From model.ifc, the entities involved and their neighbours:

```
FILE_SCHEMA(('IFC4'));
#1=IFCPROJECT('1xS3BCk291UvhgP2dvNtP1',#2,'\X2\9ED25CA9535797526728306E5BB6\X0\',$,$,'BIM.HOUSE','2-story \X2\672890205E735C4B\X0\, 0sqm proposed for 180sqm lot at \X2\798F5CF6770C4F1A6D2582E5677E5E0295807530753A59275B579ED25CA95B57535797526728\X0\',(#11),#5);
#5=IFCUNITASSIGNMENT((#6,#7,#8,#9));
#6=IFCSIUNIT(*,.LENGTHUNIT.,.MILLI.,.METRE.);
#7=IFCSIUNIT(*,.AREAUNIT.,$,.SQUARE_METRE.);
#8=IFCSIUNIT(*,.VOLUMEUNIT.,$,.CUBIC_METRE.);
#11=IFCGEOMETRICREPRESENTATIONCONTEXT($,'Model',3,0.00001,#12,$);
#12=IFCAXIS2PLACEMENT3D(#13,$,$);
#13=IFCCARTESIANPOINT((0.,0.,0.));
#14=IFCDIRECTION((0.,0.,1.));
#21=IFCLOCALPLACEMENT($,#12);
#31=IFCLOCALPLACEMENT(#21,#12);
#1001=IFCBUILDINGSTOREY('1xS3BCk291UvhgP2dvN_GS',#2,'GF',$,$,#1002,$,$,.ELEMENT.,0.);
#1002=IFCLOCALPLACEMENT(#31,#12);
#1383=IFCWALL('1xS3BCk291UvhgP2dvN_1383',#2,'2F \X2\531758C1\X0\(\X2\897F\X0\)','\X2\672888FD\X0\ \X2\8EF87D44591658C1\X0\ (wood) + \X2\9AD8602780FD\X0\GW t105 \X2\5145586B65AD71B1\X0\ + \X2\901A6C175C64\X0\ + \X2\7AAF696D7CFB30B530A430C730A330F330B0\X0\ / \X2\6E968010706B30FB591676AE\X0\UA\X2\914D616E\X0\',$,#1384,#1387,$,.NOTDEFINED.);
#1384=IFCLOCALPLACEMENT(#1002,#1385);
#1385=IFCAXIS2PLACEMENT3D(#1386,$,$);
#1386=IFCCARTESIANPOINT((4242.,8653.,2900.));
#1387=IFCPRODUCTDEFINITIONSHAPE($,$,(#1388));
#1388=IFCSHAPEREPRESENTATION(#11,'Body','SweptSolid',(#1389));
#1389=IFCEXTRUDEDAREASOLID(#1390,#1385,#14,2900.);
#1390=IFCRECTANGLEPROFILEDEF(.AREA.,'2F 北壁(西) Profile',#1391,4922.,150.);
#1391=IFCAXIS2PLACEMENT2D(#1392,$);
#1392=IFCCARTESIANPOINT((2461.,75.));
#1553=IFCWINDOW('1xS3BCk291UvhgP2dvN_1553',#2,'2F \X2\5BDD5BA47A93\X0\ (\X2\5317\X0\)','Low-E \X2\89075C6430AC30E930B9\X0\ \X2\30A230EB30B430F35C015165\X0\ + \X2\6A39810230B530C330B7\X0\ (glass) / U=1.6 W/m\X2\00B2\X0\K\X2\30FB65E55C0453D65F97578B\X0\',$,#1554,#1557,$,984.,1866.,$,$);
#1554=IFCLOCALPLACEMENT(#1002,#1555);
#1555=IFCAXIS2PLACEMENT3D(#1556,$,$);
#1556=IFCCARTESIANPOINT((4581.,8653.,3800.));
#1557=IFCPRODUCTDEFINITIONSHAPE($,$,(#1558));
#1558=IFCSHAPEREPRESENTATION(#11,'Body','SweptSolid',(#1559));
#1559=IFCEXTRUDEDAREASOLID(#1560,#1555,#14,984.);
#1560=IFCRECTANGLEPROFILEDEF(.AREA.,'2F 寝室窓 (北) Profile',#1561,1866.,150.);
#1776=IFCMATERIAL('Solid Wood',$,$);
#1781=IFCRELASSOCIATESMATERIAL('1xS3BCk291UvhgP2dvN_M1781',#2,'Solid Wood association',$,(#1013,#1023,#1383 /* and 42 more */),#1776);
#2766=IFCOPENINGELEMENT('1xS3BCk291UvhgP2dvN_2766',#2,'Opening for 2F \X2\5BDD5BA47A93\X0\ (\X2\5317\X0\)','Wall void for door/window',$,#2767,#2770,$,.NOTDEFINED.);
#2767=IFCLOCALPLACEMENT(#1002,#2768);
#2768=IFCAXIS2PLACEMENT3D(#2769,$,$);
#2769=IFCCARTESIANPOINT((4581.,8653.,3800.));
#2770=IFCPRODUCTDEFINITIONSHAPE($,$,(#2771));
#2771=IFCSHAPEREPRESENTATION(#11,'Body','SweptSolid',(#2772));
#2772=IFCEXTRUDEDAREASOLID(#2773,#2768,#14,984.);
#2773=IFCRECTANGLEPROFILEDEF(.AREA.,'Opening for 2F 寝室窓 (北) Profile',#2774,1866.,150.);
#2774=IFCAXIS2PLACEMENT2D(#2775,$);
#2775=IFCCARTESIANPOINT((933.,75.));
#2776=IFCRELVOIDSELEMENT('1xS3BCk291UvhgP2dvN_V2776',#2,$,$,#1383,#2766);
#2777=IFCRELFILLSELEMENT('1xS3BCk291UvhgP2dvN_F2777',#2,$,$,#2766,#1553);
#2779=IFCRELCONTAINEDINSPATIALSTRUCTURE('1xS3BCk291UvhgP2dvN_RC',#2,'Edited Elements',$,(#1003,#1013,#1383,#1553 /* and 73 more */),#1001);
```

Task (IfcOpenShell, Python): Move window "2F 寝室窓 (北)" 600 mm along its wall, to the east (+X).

```python
import ifcopenshell
import ifcopenshell.api.geometry
import ifcopenshell.util.placement
import ifcopenshell.util.unit

model = ifcopenshell.open("model.ifc")
unit_scale = ifcopenshell.util.unit.calculate_unit_scale(model)

window = model.by_id(1553)
opening = window.FillsVoids[0].RelatingOpeningElement
wall = opening.VoidsElements[0].RelatingBuildingElement

wall_matrix = ifcopenshell.util.placement.get_local_placement(wall.ObjectPlacement)
shift = wall_matrix[:3, 0] * 0.6 / unit_scale
before = ifcopenshell.util.placement.get_local_placement(window.ObjectPlacement)[:3, 3].copy()

# The window is not placed relative to its opening, so move both.
for product in (opening, window):
    matrix = ifcopenshell.util.placement.get_local_placement(product.ObjectPlacement)
    matrix[:3, 3] += shift
    ifcopenshell.api.geometry.edit_object_placement(model, product=product, matrix=matrix, is_si=False)

after = ifcopenshell.util.placement.get_local_placement(window.ObjectPlacement)[:3, 3]
print("window moved by", (after - before).round(3) + 0.0)

model.write("model_updated.ifc")
```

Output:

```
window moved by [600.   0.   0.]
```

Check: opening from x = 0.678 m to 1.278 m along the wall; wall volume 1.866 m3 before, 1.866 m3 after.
